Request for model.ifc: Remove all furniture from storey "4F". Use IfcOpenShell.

First a look at what the model holds.

```python
import ifcopenshell
import ifcopenshell.util.element

model = ifcopenshell.open("model.ifc")
print(model.schema)
storey = next(s for s in model.by_type("IfcBuildingStorey") if s.Name == "4F")
furniture = [e for e in ifcopenshell.util.element.get_decomposition(storey) if e.is_a("IfcFurnishingElement")]
seen = {}
for e in furniture:
    element_type = ifcopenshell.util.element.get_type(e)
    name = element_type.Name if element_type not in (None, e) else None
    seen[name] = seen.get(name, 0) + 1
for name, count in sorted(seen.items(), key=str):
    print(count, "x", name)
```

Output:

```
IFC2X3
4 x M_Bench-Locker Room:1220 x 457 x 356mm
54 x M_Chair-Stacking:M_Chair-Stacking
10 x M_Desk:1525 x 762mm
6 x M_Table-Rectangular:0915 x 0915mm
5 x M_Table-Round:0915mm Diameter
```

```python
import ifcopenshell
import ifcopenshell.api.root
import ifcopenshell.util.element

model = ifcopenshell.open("model.ifc")

storey = next(s for s in model.by_type("IfcBuildingStorey") if s.Name == "4F")
furniture = [e for e in ifcopenshell.util.element.get_decomposition(storey) if e.is_a("IfcFurnishingElement")]

for e in furniture:
    ifcopenshell.api.root.remove_product(model, product=e)
print(len(furniture), "removed")

model.write("model-out.ifc")
```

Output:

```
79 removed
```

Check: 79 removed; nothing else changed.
